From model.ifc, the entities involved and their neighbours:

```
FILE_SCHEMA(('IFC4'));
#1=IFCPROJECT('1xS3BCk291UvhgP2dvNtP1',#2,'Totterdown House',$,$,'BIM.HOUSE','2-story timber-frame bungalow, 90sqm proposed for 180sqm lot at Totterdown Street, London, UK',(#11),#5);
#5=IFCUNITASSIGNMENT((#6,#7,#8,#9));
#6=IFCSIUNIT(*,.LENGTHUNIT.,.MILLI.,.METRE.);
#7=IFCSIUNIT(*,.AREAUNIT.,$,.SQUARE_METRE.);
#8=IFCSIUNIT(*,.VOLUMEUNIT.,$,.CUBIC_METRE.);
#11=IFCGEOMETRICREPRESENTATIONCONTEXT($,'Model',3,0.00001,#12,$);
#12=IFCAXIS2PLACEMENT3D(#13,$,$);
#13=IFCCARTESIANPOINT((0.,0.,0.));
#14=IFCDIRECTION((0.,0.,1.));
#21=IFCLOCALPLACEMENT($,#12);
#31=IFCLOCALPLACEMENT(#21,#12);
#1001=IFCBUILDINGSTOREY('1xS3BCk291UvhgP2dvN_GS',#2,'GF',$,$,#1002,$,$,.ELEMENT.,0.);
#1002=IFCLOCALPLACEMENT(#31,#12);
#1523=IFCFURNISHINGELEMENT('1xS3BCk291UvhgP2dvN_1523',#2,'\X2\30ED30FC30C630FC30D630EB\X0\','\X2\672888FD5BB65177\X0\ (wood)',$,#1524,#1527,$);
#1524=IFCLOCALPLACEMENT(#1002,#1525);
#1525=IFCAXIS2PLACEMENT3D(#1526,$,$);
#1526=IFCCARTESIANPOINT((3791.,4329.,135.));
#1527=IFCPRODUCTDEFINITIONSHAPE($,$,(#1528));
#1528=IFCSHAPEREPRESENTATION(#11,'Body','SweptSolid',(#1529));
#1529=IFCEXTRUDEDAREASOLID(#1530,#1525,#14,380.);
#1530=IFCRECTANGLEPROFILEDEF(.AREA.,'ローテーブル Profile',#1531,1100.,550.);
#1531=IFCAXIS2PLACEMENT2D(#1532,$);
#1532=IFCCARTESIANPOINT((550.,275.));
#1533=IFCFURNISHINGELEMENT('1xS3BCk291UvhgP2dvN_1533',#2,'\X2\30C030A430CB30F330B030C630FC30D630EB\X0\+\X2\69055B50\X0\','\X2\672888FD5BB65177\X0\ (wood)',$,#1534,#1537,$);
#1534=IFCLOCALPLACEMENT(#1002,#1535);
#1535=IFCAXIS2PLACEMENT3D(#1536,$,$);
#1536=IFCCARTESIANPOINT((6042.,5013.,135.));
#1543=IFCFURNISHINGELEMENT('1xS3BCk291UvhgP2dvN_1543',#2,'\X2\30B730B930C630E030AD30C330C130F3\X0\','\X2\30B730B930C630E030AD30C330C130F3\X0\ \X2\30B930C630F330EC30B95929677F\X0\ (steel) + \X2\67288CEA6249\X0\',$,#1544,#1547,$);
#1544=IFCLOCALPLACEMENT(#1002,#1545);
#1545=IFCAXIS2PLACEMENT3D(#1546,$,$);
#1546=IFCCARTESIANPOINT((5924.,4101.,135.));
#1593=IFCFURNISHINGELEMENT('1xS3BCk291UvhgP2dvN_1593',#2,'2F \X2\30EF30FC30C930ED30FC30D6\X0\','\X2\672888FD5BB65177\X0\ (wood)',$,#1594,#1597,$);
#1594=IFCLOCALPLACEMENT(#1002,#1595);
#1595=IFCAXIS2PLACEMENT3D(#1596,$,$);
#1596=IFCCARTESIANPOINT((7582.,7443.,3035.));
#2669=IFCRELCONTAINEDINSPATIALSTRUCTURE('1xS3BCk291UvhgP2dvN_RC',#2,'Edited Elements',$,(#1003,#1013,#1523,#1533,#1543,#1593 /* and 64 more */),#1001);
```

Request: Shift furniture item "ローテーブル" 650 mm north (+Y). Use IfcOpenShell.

```python
import ifcopenshell
import ifcopenshell.api.geometry
import ifcopenshell.util.placement

model = ifcopenshell.open("model.ifc")

item = model.by_guid("1xS3BCk291UvhgP2dvN_1523")
matrix = ifcopenshell.util.placement.get_local_placement(item.ObjectPlacement)
matrix[1, 3] += 650.0
ifcopenshell.api.geometry.edit_object_placement(model, product=item, matrix=matrix, is_si=False)

print(ifcopenshell.util.placement.get_local_placement(item.ObjectPlacement).round(3) + 0.0)

model.write("model-out.ifc")
```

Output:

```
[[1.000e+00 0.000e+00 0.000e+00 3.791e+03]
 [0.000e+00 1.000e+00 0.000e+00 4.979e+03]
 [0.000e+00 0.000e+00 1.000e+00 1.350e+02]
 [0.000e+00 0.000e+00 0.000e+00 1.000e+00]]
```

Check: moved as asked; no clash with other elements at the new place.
